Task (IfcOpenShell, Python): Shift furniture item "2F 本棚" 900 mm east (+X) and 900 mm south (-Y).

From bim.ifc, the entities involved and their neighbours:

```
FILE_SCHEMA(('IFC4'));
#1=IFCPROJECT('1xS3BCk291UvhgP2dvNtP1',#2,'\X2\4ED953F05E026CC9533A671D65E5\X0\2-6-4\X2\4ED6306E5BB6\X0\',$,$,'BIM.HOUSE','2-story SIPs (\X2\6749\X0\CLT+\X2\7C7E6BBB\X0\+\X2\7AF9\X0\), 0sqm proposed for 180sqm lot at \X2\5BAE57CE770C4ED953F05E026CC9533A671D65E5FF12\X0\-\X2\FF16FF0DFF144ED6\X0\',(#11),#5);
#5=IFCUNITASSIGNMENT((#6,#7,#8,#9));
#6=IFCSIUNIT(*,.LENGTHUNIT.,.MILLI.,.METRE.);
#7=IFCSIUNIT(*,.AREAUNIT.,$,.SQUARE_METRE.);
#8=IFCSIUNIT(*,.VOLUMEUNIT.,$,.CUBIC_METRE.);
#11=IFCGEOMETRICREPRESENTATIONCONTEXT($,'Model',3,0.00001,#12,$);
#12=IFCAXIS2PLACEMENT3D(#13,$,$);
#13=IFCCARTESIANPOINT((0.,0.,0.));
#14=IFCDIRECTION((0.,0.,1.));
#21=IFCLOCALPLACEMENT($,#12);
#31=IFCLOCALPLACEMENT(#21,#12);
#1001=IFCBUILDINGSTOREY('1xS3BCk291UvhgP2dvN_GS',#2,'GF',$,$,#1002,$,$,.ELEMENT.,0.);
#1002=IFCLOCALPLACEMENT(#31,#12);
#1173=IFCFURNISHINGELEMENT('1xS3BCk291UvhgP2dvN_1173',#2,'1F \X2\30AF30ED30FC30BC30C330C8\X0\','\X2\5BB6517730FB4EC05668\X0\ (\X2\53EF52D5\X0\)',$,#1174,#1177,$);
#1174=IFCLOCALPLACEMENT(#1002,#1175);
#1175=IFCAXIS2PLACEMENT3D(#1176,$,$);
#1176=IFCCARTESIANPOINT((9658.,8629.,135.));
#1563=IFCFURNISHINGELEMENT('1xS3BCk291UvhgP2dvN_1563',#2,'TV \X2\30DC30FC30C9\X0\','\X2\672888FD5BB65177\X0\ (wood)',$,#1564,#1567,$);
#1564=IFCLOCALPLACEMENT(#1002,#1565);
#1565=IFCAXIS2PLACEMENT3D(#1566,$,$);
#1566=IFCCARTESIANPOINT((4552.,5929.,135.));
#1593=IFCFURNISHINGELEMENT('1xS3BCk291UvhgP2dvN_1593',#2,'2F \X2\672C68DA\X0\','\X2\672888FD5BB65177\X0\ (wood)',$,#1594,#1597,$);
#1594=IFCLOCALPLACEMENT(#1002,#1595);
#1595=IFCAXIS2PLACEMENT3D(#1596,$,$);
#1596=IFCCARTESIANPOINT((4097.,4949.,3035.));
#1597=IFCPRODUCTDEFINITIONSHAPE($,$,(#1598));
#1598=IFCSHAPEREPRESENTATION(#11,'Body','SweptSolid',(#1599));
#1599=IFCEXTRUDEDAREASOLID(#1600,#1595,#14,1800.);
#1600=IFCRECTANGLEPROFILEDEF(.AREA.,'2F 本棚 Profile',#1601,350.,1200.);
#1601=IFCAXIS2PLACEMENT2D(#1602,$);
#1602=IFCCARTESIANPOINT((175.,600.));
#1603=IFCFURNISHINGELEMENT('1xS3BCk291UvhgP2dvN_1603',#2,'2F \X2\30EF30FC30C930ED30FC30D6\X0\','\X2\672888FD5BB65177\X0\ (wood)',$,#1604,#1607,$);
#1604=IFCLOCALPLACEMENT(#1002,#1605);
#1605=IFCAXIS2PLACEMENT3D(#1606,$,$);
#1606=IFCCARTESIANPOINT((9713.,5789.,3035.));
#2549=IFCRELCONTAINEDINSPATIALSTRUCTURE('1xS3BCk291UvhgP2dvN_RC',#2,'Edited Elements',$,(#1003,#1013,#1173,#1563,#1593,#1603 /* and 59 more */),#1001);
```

```python
import ifcopenshell
import ifcopenshell.api.geometry
import ifcopenshell.util.placement
import ifcopenshell.util.unit

model = ifcopenshell.open("bim.ifc")
unit_scale = ifcopenshell.util.unit.calculate_unit_scale(model)

item = model.by_guid("1xS3BCk291UvhgP2dvN_1593")
matrix = ifcopenshell.util.placement.get_local_placement(item.ObjectPlacement)
matrix[0, 3] += 0.9 / unit_scale
matrix[1, 3] -= 0.9 / unit_scale
ifcopenshell.api.geometry.edit_object_placement(model, product=item, matrix=matrix, is_si=False)

print(ifcopenshell.util.placement.get_local_placement(item.ObjectPlacement).round(3) + 0.0)

model.write("bim_edited.ifc")
```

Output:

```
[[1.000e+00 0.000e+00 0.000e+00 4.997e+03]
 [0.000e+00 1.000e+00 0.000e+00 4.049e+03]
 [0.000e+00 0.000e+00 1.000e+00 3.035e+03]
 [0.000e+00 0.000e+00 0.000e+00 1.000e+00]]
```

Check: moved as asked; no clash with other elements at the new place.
